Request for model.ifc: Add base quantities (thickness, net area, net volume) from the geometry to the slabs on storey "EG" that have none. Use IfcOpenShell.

First a look at what the model holds.

```python
import ifcopenshell
import ifcopenshell.util.element
import ifcopenshell.util.unit

model = ifcopenshell.open("model.ifc")
print(model.schema)
for unit_type in ("LENGTHUNIT", "AREAUNIT", "VOLUMEUNIT"):
    print(unit_type, ifcopenshell.util.unit.calculate_unit_scale(model, unit_type))
storey = next(s for s in model.by_type("IfcBuildingStorey") if s.Name == "EG")
slabs = [e for e in ifcopenshell.util.element.get_decomposition(storey) if e.is_a("IfcSlab")]
for e in sorted(slabs, key=lambda e: e.id()):
    print(e.id(), e.is_a(), e.Name, list(ifcopenshell.util.element.get_psets(e, qtos_only=True)), sep=" | ")
```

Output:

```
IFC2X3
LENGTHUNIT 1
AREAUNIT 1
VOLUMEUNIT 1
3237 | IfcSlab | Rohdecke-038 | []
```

```python
import ifcopenshell
import ifcopenshell.api.pset
import ifcopenshell.geom
import ifcopenshell.util.element
import ifcopenshell.util.shape
import ifcopenshell.util.unit

model = ifcopenshell.open("model.ifc")
unit_scale = ifcopenshell.util.unit.calculate_unit_scale(model)
area_scale = ifcopenshell.util.unit.calculate_unit_scale(model, "AREAUNIT")
volume_scale = ifcopenshell.util.unit.calculate_unit_scale(model, "VOLUMEUNIT")
settings = ifcopenshell.geom.settings()

storey = next(s for s in model.by_type("IfcBuildingStorey") if s.Name == "EG")
slabs = [e for e in ifcopenshell.util.element.get_decomposition(storey) if e.is_a("IfcSlab")]

for e in sorted(slabs, key=lambda e: e.id()):
    if ifcopenshell.util.element.get_psets(e, qtos_only=True, should_inherit=False):
        continue
    # Geometry comes back in metres, in the element's own axes.
    shape = ifcopenshell.geom.create_shape(settings, e)
    values = {
        "Width": ifcopenshell.util.shape.get_z(shape.geometry) / unit_scale,
        "NetArea": ifcopenshell.util.shape.get_footprint_area(shape.geometry) / area_scale,
        "NetVolume": ifcopenshell.util.shape.get_volume(shape.geometry) / volume_scale,
    }
    qto = ifcopenshell.api.pset.add_qto(model, product=e, name="BaseQuantities")
    ifcopenshell.api.pset.edit_qto(model, qto=qto, properties=values)
    print(e.id(), {k: round(v, 3) for k, v in values.items()})

model.write("model_edited.ifc")
```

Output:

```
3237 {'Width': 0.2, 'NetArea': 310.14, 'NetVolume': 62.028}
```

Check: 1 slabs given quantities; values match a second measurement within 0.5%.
